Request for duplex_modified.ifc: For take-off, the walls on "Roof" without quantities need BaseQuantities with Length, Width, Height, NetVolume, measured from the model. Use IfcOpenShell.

First a look at what the model holds.

```python
import ifcopenshell
import ifcopenshell.util.element
import ifcopenshell.util.unit

model = ifcopenshell.open("duplex_modified.ifc")
print(model.schema)
for unit_type in ("LENGTHUNIT", "AREAUNIT", "VOLUMEUNIT"):
    print(unit_type, ifcopenshell.util.unit.calculate_unit_scale(model, unit_type))
storey = next(s for s in model.by_type("IfcBuildingStorey") if s.Name == "Roof")
walls = [e for e in ifcopenshell.util.element.get_decomposition(storey) if e.is_a("IfcWall")]
for e in sorted(walls, key=lambda e: e.id()):
    print(e.id(), e.is_a(), e.Name, list(ifcopenshell.util.element.get_psets(e, qtos_only=True)), sep=" | ")
```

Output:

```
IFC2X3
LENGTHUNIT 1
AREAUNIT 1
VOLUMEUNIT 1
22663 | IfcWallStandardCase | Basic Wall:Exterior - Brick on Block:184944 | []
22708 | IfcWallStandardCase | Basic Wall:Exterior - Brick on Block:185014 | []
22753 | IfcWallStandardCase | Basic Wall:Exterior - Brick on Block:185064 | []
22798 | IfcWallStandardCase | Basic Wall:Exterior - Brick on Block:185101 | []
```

```python
import ifcopenshell
import ifcopenshell.api.pset
import ifcopenshell.geom
import ifcopenshell.util.element
import ifcopenshell.util.shape
import ifcopenshell.util.unit

model = ifcopenshell.open("duplex_modified.ifc")
unit_scale = ifcopenshell.util.unit.calculate_unit_scale(model)
volume_scale = ifcopenshell.util.unit.calculate_unit_scale(model, "VOLUMEUNIT")
settings = ifcopenshell.geom.settings()

storey = next(s for s in model.by_type("IfcBuildingStorey") if s.Name == "Roof")
walls = [e for e in ifcopenshell.util.element.get_decomposition(storey) if e.is_a("IfcWall")]

for e in sorted(walls, key=lambda e: e.id()):
    if ifcopenshell.util.element.get_psets(e, qtos_only=True, should_inherit=False):
        continue
    # Geometry comes back in metres, in the element's own axes.
    shape = ifcopenshell.geom.create_shape(settings, e)
    values = {
        "Length": ifcopenshell.util.shape.get_x(shape.geometry) / unit_scale,
        "Width": ifcopenshell.util.shape.get_y(shape.geometry) / unit_scale,
        "Height": ifcopenshell.util.shape.get_z(shape.geometry) / unit_scale,
        "NetVolume": ifcopenshell.util.shape.get_volume(shape.geometry) / volume_scale,
    }
    qto = ifcopenshell.api.pset.add_qto(model, product=e, name="BaseQuantities")
    ifcopenshell.api.pset.edit_qto(model, qto=qto, properties=values)
    print(e.id(), {k: round(v, 3) for k, v in values.items()})

model.write("duplex_modified_edited.ifc")
```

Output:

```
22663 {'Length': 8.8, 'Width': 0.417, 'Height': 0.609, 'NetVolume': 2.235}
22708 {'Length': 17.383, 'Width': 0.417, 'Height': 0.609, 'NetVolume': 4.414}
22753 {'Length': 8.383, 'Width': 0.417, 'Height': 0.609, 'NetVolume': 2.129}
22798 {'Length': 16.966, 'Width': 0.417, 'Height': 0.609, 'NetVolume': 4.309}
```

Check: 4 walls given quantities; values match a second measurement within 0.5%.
